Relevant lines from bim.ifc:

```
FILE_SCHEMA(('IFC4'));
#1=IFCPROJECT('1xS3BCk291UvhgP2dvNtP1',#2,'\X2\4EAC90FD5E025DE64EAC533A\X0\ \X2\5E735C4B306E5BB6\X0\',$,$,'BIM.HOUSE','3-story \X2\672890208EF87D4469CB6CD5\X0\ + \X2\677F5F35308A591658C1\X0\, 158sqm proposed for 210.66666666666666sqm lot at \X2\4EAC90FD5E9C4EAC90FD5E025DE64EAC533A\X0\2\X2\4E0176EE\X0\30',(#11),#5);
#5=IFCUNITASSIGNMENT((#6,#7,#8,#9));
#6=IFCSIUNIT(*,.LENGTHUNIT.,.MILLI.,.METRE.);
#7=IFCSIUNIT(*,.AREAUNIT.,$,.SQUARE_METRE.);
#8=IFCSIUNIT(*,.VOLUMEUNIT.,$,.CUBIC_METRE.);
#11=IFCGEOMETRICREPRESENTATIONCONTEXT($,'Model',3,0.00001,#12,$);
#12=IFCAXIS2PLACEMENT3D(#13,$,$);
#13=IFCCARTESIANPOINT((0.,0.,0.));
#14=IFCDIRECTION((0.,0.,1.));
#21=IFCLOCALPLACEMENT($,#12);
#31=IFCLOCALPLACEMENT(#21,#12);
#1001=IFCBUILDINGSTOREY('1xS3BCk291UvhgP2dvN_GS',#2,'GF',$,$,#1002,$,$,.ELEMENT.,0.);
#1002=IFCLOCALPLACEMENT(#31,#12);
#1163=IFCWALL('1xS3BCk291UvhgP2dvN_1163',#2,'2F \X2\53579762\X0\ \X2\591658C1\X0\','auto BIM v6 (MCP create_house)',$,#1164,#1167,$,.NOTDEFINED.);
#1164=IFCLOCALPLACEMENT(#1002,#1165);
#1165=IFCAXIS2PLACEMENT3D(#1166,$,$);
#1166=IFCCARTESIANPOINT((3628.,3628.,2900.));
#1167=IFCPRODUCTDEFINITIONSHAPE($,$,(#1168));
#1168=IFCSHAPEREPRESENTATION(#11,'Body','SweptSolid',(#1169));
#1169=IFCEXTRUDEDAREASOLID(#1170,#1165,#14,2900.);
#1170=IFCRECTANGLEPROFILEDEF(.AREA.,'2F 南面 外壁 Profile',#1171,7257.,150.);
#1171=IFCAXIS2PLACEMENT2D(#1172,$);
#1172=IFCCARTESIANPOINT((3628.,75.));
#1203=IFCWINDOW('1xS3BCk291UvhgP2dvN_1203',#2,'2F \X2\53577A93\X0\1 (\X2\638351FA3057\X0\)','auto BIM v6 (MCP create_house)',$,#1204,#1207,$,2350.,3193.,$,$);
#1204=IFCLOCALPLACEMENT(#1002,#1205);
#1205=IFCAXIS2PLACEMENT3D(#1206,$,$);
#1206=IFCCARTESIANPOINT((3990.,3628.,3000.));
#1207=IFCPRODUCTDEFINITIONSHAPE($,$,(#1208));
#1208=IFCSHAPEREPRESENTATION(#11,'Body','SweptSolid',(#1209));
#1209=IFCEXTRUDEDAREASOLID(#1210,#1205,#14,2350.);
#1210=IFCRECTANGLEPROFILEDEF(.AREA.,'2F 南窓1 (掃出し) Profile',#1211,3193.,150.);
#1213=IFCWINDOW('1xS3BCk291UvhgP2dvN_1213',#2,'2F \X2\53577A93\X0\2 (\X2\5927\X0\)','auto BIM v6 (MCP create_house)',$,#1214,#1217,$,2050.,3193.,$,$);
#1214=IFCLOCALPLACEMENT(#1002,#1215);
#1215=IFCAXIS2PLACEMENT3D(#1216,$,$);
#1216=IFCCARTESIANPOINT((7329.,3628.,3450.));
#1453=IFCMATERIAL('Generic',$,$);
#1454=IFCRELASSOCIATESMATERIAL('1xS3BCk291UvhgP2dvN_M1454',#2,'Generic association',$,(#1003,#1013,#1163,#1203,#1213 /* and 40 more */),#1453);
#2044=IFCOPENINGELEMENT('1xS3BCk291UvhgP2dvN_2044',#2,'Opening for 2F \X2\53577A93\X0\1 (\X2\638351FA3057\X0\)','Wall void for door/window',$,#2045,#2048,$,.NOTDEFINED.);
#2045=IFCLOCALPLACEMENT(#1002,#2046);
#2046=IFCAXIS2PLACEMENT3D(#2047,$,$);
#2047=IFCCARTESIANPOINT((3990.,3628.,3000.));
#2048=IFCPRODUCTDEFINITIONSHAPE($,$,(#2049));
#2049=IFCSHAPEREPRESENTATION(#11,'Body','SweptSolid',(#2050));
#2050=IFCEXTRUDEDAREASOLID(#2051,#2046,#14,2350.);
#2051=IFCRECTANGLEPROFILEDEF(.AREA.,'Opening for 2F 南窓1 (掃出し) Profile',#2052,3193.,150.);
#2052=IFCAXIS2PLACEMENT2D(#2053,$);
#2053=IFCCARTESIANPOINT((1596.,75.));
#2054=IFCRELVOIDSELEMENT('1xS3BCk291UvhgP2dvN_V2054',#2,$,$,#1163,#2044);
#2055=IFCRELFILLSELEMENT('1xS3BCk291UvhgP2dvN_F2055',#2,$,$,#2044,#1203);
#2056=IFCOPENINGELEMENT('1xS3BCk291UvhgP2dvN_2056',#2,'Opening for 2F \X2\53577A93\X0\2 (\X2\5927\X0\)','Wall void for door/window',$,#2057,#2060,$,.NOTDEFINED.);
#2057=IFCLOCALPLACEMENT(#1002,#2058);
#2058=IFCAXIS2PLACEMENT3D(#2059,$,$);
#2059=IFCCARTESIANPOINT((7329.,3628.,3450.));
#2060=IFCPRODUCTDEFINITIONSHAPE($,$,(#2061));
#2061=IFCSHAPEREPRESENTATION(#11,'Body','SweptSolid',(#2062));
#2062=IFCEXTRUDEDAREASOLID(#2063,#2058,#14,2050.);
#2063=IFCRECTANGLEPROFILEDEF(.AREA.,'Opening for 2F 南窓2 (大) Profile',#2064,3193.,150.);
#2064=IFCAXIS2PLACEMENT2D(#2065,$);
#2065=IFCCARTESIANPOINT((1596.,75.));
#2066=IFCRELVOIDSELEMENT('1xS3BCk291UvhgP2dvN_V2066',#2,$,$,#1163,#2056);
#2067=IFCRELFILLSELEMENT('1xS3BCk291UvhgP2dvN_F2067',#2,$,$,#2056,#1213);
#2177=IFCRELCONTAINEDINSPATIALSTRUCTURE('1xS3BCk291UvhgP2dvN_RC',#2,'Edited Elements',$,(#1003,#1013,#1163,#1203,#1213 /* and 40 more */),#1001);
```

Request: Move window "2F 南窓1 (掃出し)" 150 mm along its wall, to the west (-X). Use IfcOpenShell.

```python
import ifcopenshell
import ifcopenshell.api.geometry
import ifcopenshell.util.placement
import ifcopenshell.util.unit

model = ifcopenshell.open("bim.ifc")
unit_scale = ifcopenshell.util.unit.calculate_unit_scale(model)

window = model.by_id(1203)
opening = window.FillsVoids[0].RelatingOpeningElement
wall = opening.VoidsElements[0].RelatingBuildingElement

wall_matrix = ifcopenshell.util.placement.get_local_placement(wall.ObjectPlacement)
shift = wall_matrix[:3, 0] * -0.15 / unit_scale
before = ifcopenshell.util.placement.get_local_placement(window.ObjectPlacement)[:3, 3].copy()

# The window is not placed relative to its opening, so move both.
for product in (opening, window):
    matrix = ifcopenshell.util.placement.get_local_placement(product.ObjectPlacement)
    matrix[:3, 3] += shift
    ifcopenshell.api.geometry.edit_object_placement(model, product=product, matrix=matrix, is_si=False)

after = ifcopenshell.util.placement.get_local_placement(window.ObjectPlacement)[:3, 3]
print("window moved by", (after - before).round(3) + 0.0)

model.write("bim_rev.ifc")
```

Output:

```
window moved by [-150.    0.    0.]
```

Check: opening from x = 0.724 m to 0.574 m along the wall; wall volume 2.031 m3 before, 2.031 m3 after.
